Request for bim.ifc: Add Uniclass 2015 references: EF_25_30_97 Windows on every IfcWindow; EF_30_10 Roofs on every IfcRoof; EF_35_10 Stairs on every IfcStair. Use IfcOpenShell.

First a look at what the model holds.

```python
import ifcopenshell

model = ifcopenshell.open("bim.ifc")
print(model.schema)
print("classifications:", [c.Name for c in model.by_type("IfcClassification")])
for ifc_class in ("IfcDoor", "IfcRoof", "IfcStair", "IfcWall", "IfcWindow"):
    print(ifc_class, len(model.by_type(ifc_class)))
```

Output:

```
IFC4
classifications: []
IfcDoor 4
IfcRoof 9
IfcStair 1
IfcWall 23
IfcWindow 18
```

```python
import ifcopenshell
import ifcopenshell.api.classification

model = ifcopenshell.open("bim.ifc")

system = ifcopenshell.api.classification.add_classification(model, classification="Uniclass 2015")

codes = {
    "IfcWindow": ("EF_25_30_97", "Windows"),
    "IfcRoof": ("EF_30_10", "Roofs"),
    "IfcStair": ("EF_35_10", "Stairs"),
}
for ifc_class, (code, name) in codes.items():
    products = model.by_type(ifc_class)
    ifcopenshell.api.classification.add_reference(
        model, products=products, classification=system, identification=code, name=name
    )
    print(code, len(products))

model.write("bim_rev.ifc")
```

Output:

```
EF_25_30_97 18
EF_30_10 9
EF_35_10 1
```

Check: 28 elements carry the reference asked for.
